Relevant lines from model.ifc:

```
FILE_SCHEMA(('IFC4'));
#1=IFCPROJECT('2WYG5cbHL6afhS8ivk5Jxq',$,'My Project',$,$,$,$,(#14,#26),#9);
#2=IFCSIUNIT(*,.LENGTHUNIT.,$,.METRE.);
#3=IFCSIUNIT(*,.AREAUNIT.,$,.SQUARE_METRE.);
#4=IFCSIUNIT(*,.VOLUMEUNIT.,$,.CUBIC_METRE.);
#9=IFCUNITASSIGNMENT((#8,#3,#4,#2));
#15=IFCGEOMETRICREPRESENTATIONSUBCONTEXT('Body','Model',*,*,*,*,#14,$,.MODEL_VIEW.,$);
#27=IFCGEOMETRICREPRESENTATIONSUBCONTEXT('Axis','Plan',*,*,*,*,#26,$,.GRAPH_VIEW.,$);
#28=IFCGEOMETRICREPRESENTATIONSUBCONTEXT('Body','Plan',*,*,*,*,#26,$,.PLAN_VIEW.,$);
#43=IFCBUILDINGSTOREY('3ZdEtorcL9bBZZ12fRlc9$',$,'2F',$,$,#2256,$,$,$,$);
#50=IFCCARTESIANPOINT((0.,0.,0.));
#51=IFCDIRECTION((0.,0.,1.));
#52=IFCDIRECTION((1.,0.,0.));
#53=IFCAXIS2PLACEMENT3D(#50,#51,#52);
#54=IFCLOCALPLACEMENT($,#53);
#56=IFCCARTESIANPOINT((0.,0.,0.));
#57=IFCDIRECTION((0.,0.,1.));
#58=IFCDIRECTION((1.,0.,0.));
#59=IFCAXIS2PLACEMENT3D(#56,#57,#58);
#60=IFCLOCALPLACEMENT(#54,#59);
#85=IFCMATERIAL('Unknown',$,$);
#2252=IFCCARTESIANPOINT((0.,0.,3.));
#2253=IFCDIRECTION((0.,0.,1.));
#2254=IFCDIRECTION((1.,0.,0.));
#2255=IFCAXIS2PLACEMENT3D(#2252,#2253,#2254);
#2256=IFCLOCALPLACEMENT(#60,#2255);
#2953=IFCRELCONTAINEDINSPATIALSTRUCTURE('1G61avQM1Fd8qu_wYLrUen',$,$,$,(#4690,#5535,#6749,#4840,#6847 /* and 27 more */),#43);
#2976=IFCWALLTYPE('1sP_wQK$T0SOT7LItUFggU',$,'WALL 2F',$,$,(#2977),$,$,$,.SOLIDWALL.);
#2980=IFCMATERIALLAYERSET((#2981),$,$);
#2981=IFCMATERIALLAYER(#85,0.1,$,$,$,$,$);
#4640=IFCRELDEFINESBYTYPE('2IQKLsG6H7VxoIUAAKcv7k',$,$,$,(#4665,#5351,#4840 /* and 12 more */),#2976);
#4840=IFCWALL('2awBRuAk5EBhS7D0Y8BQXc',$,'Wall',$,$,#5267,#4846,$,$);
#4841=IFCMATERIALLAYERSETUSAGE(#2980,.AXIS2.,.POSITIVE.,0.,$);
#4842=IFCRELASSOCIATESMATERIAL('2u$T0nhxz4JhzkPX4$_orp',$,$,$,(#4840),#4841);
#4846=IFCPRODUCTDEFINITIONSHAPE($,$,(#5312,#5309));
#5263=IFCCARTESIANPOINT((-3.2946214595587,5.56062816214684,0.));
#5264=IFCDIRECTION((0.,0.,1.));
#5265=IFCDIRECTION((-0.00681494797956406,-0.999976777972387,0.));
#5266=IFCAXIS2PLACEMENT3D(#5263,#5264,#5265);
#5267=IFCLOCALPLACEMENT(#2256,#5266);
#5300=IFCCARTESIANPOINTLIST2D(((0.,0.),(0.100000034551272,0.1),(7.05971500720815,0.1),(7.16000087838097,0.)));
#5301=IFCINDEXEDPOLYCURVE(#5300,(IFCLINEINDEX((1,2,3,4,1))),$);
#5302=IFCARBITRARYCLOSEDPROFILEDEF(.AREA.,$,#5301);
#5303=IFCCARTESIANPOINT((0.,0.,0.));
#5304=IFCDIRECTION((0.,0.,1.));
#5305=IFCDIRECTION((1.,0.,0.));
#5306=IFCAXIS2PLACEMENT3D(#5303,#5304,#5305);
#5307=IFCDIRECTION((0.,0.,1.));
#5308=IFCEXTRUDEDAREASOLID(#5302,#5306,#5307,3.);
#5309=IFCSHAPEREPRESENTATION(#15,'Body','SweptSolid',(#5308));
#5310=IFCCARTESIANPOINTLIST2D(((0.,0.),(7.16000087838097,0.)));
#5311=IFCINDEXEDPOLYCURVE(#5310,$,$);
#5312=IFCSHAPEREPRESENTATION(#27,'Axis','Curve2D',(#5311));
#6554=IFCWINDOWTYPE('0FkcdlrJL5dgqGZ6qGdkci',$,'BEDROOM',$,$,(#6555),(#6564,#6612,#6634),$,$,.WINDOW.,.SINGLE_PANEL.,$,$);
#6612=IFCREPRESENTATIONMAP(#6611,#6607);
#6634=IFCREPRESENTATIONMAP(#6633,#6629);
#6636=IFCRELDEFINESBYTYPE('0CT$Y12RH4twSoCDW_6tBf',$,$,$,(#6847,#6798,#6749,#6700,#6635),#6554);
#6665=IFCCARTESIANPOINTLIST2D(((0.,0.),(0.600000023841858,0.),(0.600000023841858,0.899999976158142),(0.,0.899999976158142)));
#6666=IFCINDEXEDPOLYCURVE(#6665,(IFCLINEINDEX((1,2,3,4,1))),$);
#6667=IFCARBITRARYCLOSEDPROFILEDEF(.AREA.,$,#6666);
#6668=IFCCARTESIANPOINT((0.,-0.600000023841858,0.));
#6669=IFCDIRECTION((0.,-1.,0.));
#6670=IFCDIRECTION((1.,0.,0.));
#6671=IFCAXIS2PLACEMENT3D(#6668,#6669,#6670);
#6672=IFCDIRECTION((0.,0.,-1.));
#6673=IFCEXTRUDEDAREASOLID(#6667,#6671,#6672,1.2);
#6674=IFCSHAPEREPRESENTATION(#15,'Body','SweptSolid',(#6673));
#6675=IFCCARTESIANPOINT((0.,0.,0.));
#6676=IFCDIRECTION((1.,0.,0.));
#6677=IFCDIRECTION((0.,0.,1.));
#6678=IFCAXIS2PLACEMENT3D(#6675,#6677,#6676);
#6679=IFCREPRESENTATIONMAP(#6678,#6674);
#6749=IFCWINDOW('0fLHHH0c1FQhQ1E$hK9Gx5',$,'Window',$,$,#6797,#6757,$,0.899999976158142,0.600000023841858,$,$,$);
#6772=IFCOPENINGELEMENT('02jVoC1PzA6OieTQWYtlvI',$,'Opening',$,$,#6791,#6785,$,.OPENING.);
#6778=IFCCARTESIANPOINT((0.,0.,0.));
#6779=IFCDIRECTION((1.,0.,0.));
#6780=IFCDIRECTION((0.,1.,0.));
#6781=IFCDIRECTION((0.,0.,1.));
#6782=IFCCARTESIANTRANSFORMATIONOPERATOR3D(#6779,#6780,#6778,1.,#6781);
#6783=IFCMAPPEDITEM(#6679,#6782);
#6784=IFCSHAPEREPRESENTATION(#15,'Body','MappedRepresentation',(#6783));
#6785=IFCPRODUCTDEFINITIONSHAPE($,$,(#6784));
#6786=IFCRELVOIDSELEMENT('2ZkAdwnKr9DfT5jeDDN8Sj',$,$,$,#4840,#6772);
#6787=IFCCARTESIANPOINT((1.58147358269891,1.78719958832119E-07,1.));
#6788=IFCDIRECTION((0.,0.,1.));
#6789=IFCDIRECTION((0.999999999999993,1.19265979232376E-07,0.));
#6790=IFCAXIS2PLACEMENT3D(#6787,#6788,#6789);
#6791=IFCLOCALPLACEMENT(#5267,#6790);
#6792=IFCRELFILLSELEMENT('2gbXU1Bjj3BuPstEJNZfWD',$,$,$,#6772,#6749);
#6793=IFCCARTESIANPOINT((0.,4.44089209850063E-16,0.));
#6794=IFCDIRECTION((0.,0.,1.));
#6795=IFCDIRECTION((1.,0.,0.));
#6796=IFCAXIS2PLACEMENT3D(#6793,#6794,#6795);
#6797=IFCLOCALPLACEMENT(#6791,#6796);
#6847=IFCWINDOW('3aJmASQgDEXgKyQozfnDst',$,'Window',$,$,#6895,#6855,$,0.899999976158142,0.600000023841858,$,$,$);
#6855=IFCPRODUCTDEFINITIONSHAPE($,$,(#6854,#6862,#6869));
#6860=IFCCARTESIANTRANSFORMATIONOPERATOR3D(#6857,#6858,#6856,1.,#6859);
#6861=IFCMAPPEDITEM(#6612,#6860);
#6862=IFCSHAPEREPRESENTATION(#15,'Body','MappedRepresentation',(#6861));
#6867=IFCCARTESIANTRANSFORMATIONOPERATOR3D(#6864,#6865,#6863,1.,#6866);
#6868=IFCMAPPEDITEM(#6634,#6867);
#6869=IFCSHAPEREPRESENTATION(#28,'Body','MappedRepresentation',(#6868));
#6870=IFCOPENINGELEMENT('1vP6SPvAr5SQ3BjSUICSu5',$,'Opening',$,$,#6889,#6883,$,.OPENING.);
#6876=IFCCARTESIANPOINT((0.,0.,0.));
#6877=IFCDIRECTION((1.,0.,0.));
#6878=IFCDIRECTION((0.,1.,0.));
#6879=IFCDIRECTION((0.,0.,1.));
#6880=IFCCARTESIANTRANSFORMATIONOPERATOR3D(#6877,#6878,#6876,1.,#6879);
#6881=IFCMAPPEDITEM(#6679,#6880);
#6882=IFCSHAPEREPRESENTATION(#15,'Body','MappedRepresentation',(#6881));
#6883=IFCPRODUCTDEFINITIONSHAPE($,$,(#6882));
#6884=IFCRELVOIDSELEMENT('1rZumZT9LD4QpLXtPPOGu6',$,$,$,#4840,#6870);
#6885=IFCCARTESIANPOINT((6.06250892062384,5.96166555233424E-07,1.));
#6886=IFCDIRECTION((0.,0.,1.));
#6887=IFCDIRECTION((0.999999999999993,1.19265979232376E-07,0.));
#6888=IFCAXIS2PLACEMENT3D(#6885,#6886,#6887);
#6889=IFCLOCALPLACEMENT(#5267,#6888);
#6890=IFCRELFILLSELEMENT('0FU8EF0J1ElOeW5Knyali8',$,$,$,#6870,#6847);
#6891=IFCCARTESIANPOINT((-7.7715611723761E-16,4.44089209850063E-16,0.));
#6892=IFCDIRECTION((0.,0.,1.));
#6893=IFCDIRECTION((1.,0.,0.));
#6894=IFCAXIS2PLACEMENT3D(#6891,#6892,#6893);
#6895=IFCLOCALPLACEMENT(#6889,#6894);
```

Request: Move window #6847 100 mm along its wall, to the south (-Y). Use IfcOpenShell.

```python
import ifcopenshell
import ifcopenshell.api.geometry
import ifcopenshell.util.placement

model = ifcopenshell.open("model.ifc")

window = model.by_id(6847)
opening = window.FillsVoids[0].RelatingOpeningElement
wall = opening.VoidsElements[0].RelatingBuildingElement

wall_matrix = ifcopenshell.util.placement.get_local_placement(wall.ObjectPlacement)
shift = wall_matrix[:3, 0] * 0.1
before = ifcopenshell.util.placement.get_local_placement(window.ObjectPlacement)[:3, 3].copy()

# The window is placed relative to its opening, so it follows when the opening moves.
matrix = ifcopenshell.util.placement.get_local_placement(opening.ObjectPlacement)
matrix[:3, 3] += shift
ifcopenshell.api.geometry.edit_object_placement(
    model, product=opening, matrix=matrix, is_si=False, should_transform_children=True
)

after = ifcopenshell.util.placement.get_local_placement(window.ObjectPlacement)[:3, 3]
print("window moved by", (after - before).round(3) + 0.0)

model.write("model-out.ifc")
```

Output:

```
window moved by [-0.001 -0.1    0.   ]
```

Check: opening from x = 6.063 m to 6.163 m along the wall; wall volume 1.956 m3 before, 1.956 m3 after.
